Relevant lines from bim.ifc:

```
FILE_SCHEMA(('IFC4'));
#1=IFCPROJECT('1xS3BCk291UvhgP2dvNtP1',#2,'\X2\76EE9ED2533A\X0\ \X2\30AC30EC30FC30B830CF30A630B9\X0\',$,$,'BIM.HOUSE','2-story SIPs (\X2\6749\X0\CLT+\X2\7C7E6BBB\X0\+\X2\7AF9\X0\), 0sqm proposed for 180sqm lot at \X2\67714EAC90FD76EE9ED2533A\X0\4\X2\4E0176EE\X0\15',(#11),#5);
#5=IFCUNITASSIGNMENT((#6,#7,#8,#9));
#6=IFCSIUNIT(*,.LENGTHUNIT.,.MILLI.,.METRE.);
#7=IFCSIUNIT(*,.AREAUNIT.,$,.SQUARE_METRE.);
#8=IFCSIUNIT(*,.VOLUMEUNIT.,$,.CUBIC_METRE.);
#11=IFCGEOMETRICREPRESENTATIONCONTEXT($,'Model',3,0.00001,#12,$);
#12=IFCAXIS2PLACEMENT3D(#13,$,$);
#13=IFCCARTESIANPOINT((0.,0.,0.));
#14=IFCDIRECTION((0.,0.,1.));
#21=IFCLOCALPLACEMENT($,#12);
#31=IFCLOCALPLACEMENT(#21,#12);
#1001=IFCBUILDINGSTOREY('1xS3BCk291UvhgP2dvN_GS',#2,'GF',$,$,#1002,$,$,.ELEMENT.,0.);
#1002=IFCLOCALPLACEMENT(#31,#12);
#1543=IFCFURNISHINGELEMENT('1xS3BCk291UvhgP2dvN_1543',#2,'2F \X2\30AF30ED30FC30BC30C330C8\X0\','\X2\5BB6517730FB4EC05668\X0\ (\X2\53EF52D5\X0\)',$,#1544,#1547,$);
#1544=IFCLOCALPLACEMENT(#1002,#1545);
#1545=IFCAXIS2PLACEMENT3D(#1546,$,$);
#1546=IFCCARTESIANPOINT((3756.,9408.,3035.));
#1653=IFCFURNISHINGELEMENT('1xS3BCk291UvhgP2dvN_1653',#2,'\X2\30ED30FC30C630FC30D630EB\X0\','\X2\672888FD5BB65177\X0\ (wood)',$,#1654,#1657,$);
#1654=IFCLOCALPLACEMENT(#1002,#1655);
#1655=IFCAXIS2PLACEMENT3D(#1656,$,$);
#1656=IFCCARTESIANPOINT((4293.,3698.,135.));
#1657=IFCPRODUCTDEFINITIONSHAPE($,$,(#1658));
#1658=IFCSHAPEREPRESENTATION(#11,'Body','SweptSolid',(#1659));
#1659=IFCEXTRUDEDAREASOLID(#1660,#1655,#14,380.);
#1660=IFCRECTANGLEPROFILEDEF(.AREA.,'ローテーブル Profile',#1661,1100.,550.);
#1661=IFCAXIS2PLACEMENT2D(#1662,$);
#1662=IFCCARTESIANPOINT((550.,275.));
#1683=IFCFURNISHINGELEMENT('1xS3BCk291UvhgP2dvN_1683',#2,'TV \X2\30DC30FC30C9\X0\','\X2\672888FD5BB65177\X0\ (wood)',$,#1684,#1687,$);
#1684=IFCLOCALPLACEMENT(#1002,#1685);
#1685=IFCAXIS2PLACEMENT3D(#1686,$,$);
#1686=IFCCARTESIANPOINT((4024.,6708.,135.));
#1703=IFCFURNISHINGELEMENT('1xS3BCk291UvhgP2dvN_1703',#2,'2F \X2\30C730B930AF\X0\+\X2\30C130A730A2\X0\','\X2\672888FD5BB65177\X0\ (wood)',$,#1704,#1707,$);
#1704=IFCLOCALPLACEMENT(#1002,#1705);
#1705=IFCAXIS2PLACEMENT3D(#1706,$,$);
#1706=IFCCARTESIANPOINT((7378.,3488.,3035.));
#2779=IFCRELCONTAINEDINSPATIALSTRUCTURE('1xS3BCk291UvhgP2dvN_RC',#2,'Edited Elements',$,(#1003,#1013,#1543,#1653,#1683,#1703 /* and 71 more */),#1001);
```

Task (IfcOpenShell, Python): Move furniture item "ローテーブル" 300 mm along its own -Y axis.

```python
import ifcopenshell
import ifcopenshell.api.geometry
import ifcopenshell.util.placement
import ifcopenshell.util.unit

model = ifcopenshell.open("bim.ifc")
unit_scale = ifcopenshell.util.unit.calculate_unit_scale(model)

item = model.by_guid("1xS3BCk291UvhgP2dvN_1653")
matrix = ifcopenshell.util.placement.get_local_placement(item.ObjectPlacement)
matrix[:3, 3] -= matrix[:3, 1] * 0.3 / unit_scale
ifcopenshell.api.geometry.edit_object_placement(model, product=item, matrix=matrix, is_si=False)

print(ifcopenshell.util.placement.get_local_placement(item.ObjectPlacement).round(3) + 0.0)

model.write("bim_v2.ifc")
```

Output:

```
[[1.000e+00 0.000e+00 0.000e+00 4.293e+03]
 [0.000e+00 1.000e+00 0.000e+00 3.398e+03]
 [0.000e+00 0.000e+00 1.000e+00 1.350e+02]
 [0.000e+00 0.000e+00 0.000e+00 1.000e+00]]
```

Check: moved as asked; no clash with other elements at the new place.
